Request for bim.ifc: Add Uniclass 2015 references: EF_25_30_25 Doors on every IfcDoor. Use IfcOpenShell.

First a look at what the model holds.

```python
import ifcopenshell

model = ifcopenshell.open("bim.ifc")
print(model.schema)
print("classifications:", [c.Name for c in model.by_type("IfcClassification")])
for ifc_class in ("IfcDoor", "IfcRoof", "IfcStair", "IfcWall", "IfcWindow"):
    print(ifc_class, len(model.by_type(ifc_class)))
```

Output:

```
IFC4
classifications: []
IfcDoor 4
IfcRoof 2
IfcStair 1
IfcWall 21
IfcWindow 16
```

```python
import ifcopenshell
import ifcopenshell.api.classification

model = ifcopenshell.open("bim.ifc")

system = ifcopenshell.api.classification.add_classification(model, classification="Uniclass 2015")

codes = {
    "IfcDoor": ("EF_25_30_25", "Doors"),
}
for ifc_class, (code, name) in codes.items():
    products = model.by_type(ifc_class)
    ifcopenshell.api.classification.add_reference(
        model, products=products, classification=system, identification=code, name=name
    )
    print(code, len(products))

model.write("bim_v2.ifc")
```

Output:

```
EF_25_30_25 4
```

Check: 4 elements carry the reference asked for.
